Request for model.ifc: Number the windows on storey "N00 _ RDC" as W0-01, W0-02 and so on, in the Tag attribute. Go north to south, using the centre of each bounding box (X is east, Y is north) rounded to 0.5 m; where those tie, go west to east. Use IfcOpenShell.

First a look at what the model holds.

```python
import ifcopenshell
import ifcopenshell.util.element
import ifcopenshell.util.placement

model = ifcopenshell.open("model.ifc")
print(model.schema)
storey = next(s for s in model.by_type("IfcBuildingStorey") if s.Name == "N00 _ RDC")
windows = [e for e in ifcopenshell.util.element.get_decomposition(storey) if e.is_a("IfcWindow")]
for e in sorted(windows, key=lambda e: e.id()):
    origin = ifcopenshell.util.placement.get_local_placement(e.ObjectPlacement)[:3, 3]
    print(e.id(), e.Tag, e.Name, origin.round(2) + 0.0, sep=" | ")
```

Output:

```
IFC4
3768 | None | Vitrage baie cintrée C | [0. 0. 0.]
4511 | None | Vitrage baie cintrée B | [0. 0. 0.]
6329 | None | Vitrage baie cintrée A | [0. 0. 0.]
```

```python
import ifcopenshell
import ifcopenshell.geom
import ifcopenshell.util.element
import ifcopenshell.util.shape

model = ifcopenshell.open("model.ifc")
settings = ifcopenshell.geom.settings()
settings.set("use-world-coords", True)


def centre(element):
    shape = ifcopenshell.geom.create_shape(settings, element)
    return ifcopenshell.util.shape.get_bbox_centroid(shape.geometry)


storey = next(s for s in model.by_type("IfcBuildingStorey") if s.Name == "N00 _ RDC")
windows = [e for e in ifcopenshell.util.element.get_decomposition(storey) if e.is_a("IfcWindow")]

# Insertion points can sit at a corner or the storey origin, so sort by the geometry (in metres).
centres = {e: centre(e) for e in windows}
windows.sort(key=lambda e: (-round(centres[e][1] / 0.5), centres[e][0]))

for i, e in enumerate(windows, start=1):
    number = f"W0-{i:02d}"
    e.Tag = number
    print(e.id(), number)

model.write("model_rev.ifc")
```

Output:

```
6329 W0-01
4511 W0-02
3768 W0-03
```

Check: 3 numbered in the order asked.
